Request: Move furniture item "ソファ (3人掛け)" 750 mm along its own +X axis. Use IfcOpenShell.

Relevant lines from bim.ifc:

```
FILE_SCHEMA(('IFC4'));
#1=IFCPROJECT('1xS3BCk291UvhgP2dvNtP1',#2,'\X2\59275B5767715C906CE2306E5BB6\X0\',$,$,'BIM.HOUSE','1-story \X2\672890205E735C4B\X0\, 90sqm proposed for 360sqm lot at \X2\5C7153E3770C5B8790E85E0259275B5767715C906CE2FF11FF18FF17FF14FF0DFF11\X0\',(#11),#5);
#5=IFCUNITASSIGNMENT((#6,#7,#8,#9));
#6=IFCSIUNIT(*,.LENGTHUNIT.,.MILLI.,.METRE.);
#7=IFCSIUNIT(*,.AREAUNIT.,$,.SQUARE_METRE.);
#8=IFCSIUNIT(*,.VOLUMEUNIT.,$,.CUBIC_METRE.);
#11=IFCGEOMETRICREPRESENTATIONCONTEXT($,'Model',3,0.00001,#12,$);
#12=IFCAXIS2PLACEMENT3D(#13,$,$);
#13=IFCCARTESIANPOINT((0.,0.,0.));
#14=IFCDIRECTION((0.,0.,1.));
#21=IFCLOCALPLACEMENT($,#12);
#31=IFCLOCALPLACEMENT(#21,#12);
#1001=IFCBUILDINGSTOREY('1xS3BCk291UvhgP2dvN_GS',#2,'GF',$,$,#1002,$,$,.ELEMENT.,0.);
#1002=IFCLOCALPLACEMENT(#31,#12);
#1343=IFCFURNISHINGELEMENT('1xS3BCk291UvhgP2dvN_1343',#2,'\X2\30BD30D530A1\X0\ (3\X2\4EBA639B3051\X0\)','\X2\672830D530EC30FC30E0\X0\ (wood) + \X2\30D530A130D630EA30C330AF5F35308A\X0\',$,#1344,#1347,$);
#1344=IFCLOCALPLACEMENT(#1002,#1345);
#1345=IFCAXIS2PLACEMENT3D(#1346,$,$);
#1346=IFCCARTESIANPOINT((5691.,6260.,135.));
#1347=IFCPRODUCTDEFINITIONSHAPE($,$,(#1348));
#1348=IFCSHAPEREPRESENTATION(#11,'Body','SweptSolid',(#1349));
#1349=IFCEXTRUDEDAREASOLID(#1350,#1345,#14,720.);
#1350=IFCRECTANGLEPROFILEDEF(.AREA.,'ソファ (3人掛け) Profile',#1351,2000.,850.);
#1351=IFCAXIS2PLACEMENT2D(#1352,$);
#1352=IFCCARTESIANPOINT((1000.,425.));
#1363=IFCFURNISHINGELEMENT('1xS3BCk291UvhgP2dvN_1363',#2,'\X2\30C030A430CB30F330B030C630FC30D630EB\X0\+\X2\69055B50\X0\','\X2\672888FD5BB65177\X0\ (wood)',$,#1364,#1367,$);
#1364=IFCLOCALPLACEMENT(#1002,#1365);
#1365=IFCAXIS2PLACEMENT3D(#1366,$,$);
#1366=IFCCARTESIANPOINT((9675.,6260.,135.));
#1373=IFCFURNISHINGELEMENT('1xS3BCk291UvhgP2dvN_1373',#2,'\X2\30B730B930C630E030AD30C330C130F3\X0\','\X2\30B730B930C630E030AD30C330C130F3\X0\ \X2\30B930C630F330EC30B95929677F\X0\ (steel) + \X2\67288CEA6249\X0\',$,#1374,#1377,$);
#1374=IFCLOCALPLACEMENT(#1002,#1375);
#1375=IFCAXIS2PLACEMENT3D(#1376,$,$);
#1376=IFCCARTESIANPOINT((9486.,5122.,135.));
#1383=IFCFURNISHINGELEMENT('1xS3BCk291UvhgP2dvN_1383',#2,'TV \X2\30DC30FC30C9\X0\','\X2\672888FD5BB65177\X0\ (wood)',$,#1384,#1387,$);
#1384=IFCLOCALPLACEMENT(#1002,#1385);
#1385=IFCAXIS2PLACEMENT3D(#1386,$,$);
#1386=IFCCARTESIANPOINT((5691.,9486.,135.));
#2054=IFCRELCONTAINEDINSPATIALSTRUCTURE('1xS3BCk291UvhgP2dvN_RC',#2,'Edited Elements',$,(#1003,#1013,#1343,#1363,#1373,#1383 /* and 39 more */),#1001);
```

```python
import ifcopenshell
import ifcopenshell.api.geometry
import ifcopenshell.util.placement
import ifcopenshell.util.unit

model = ifcopenshell.open("bim.ifc")
unit_scale = ifcopenshell.util.unit.calculate_unit_scale(model)

item = model.by_guid("1xS3BCk291UvhgP2dvN_1343")
matrix = ifcopenshell.util.placement.get_local_placement(item.ObjectPlacement)
matrix[:3, 3] += matrix[:3, 0] * 0.75 / unit_scale
ifcopenshell.api.geometry.edit_object_placement(model, product=item, matrix=matrix, is_si=False)

print(ifcopenshell.util.placement.get_local_placement(item.ObjectPlacement).round(3) + 0.0)

model.write("bim_v2.ifc")
```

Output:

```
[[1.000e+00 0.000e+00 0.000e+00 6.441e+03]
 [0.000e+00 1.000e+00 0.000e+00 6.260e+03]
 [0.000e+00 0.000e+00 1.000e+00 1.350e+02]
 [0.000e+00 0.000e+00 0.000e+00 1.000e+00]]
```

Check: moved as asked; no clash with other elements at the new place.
